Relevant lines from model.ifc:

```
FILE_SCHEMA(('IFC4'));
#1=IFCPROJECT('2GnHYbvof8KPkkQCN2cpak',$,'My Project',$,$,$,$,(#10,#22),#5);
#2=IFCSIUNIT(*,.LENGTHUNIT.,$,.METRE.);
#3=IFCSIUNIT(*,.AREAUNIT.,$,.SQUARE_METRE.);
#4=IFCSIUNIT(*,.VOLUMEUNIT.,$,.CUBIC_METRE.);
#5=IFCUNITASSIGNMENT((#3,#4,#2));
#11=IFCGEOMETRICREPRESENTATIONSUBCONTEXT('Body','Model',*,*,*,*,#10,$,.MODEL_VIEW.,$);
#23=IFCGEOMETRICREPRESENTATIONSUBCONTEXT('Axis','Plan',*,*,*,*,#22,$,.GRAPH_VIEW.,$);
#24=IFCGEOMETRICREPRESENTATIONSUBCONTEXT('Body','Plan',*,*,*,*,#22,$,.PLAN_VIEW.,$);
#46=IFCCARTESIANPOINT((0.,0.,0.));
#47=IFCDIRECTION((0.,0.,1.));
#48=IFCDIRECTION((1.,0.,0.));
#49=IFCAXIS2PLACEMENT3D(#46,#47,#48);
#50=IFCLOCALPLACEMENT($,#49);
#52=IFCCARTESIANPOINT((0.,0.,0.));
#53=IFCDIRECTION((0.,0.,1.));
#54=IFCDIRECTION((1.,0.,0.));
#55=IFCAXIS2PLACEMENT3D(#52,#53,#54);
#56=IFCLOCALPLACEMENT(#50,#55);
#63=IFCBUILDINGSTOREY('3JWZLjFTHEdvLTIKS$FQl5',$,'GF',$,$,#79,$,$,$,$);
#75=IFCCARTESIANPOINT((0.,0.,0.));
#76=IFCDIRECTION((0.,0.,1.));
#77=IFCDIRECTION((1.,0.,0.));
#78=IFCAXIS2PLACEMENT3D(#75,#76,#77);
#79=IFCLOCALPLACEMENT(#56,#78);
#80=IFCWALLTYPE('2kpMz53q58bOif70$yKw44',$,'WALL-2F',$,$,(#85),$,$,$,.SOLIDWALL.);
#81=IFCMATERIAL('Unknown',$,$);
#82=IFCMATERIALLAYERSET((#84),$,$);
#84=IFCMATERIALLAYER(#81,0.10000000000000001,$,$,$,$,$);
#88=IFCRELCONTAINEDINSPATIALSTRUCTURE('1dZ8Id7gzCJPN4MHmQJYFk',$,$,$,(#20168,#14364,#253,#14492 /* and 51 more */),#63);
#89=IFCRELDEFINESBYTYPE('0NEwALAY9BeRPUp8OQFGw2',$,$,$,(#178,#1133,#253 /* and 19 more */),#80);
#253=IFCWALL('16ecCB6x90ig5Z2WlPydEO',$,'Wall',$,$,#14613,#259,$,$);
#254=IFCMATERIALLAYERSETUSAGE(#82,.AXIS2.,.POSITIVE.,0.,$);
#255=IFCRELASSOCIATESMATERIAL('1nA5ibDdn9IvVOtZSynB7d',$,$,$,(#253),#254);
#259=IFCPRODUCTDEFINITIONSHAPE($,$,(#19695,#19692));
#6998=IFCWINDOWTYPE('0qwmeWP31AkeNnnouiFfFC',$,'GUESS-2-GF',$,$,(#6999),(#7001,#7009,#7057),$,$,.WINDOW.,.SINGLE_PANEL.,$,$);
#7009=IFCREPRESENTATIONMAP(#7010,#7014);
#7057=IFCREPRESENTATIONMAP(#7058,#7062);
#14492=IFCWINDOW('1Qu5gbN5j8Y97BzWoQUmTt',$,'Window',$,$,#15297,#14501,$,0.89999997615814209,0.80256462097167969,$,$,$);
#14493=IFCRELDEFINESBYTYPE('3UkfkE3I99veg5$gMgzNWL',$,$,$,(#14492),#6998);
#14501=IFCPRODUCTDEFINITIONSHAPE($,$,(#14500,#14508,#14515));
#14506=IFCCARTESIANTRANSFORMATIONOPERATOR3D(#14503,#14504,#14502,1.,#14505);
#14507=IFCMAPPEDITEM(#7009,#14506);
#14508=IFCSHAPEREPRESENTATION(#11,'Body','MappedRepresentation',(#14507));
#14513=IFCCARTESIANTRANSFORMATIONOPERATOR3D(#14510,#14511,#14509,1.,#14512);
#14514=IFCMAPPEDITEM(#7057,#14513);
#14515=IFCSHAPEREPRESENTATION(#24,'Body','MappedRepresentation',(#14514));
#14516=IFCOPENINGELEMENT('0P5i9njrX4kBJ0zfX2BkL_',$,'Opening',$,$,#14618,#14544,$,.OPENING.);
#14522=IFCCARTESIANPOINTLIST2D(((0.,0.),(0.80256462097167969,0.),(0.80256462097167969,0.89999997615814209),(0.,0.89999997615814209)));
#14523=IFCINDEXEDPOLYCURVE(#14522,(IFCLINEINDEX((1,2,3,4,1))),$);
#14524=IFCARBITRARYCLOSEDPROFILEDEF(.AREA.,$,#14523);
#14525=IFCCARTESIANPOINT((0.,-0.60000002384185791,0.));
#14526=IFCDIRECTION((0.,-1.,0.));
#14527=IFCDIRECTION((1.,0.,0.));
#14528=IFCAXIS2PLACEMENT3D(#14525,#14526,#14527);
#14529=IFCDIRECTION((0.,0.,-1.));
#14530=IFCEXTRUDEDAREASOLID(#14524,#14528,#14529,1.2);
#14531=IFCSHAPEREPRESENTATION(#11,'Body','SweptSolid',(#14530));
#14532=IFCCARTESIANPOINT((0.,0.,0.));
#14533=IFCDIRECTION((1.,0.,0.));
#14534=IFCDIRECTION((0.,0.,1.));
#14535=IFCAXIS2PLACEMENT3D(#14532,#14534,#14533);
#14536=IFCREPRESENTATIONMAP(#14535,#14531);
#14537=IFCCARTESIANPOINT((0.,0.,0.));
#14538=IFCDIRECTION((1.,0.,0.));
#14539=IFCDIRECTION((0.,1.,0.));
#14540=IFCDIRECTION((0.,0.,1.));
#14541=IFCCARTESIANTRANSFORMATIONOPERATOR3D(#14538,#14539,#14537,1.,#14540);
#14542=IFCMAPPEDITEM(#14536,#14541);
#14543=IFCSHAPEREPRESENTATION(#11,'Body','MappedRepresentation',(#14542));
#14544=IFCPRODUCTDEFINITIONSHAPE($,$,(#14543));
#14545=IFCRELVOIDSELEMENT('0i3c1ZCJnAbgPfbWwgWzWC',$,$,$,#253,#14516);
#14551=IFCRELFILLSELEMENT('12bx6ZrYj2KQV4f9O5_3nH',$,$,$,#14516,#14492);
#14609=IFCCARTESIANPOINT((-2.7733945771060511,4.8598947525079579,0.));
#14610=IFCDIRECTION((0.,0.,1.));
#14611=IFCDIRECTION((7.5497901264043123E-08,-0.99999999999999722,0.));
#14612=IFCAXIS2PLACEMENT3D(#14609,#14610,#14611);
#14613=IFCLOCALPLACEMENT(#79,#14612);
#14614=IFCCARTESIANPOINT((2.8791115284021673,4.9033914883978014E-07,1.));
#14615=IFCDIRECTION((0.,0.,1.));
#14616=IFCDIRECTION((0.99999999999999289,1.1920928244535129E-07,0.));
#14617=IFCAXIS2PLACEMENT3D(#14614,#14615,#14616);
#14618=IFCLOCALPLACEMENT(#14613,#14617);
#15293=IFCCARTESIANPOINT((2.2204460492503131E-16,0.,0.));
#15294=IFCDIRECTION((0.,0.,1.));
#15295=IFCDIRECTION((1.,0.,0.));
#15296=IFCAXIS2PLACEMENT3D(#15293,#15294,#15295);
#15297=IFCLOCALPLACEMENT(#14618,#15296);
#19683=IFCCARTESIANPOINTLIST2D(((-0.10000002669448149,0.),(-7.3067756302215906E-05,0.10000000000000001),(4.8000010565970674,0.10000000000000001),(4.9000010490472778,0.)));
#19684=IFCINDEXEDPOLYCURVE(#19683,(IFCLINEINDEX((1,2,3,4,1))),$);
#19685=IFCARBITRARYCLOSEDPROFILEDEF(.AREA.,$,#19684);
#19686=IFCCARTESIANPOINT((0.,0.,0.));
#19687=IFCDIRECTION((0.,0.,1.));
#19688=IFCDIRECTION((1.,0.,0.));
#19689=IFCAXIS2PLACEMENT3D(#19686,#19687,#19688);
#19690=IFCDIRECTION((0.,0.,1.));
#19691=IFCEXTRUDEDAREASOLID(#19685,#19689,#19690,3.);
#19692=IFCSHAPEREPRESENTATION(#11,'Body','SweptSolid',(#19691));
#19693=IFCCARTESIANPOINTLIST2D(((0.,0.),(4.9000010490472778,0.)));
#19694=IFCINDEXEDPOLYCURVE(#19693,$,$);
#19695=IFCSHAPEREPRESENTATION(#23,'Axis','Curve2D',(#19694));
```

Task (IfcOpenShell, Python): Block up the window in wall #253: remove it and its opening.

```python
import ifcopenshell
import ifcopenshell.api.feature
import ifcopenshell.api.root
import ifcopenshell.geom
import ifcopenshell.util.shape

model = ifcopenshell.open("model.ifc")
settings = ifcopenshell.geom.settings()


def volume(element):
    """Net volume in cubic metres, openings subtracted."""
    shape = ifcopenshell.geom.create_shape(settings, element)
    return ifcopenshell.util.shape.get_volume(shape.geometry)


window = model.by_id(14492)
opening = window.FillsVoids[0].RelatingOpeningElement
wall = opening.VoidsElements[0].RelatingBuildingElement
before = volume(wall)

ifcopenshell.api.root.remove_product(model, product=window)
ifcopenshell.api.feature.remove_feature(model, feature=opening)

after = volume(wall)

print(f"wall volume {before:.3f} -> {after:.3f} m3")

model.write("model-out.ifc")
```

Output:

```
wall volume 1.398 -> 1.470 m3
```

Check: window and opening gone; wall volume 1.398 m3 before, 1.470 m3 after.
